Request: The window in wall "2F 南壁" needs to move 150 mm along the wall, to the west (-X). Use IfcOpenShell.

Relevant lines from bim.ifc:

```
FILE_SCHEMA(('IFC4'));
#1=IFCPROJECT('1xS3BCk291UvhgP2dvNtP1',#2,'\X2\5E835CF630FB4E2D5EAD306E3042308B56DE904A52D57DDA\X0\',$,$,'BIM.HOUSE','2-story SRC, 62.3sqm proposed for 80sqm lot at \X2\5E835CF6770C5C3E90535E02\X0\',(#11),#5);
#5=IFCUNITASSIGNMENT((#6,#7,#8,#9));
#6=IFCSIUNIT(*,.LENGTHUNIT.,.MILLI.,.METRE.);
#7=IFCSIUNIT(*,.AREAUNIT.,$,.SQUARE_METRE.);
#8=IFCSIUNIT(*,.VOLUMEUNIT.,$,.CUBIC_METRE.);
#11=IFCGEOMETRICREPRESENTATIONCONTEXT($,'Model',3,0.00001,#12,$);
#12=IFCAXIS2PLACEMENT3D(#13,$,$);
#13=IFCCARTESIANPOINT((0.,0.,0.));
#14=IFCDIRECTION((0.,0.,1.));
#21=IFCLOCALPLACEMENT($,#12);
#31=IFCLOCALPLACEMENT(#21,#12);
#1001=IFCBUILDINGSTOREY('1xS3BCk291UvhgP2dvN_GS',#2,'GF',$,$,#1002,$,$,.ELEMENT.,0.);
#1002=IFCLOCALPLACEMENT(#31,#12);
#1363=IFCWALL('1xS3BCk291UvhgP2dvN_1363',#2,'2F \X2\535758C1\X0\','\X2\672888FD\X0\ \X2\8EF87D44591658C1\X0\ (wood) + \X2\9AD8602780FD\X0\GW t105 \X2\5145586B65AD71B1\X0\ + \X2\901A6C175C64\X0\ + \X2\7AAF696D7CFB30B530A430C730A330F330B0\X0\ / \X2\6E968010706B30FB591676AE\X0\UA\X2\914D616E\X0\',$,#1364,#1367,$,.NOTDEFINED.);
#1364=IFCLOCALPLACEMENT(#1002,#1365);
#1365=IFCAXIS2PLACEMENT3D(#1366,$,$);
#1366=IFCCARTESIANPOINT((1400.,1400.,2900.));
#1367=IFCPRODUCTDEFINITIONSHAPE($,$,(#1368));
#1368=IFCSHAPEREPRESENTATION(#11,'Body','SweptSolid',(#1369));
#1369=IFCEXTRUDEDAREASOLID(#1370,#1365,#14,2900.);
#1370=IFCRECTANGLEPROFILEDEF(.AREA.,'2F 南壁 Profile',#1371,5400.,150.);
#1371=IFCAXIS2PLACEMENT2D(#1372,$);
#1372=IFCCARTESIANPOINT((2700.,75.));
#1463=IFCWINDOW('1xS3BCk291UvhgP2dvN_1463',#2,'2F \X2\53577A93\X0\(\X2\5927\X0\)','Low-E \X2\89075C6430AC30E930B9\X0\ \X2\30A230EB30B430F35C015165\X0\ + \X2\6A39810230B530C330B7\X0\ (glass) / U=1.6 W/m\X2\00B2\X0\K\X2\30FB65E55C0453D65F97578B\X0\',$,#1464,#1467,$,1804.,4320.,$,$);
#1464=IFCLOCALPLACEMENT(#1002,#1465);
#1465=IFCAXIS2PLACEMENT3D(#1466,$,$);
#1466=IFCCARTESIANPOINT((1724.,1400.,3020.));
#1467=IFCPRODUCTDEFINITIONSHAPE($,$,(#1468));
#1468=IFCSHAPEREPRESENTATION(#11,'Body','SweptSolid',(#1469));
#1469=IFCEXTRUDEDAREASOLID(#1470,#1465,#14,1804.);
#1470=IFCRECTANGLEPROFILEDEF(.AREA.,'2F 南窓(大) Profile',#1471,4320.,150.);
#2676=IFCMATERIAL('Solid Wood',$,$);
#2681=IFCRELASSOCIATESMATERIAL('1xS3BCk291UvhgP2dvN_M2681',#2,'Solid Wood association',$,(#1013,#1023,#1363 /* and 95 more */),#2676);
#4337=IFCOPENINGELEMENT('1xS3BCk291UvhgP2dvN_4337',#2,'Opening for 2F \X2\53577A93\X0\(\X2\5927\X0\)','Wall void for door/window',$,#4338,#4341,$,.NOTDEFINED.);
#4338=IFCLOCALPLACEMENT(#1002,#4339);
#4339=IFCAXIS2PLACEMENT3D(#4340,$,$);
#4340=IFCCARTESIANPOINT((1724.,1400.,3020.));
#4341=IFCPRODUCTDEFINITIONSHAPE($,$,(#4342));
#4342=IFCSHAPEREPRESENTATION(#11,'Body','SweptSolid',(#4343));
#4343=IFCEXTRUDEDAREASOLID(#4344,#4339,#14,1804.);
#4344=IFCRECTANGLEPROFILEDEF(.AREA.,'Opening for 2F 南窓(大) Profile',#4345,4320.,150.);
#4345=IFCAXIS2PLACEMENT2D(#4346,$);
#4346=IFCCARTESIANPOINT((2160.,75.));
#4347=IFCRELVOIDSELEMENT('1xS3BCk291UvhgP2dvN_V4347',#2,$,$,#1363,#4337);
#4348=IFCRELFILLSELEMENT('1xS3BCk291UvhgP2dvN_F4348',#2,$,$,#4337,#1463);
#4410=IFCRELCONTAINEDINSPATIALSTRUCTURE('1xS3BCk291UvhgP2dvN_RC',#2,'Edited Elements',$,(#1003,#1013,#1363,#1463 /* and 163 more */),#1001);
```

```python
import ifcopenshell
import ifcopenshell.api.geometry
import ifcopenshell.util.placement

model = ifcopenshell.open("bim.ifc")

window = model.by_guid("1xS3BCk291UvhgP2dvN_1463")
opening = window.FillsVoids[0].RelatingOpeningElement
wall = opening.VoidsElements[0].RelatingBuildingElement

wall_matrix = ifcopenshell.util.placement.get_local_placement(wall.ObjectPlacement)
shift = wall_matrix[:3, 0] * -150.0
before = ifcopenshell.util.placement.get_local_placement(window.ObjectPlacement)[:3, 3].copy()

# The window is not placed relative to its opening, so move both.
for product in (opening, window):
    matrix = ifcopenshell.util.placement.get_local_placement(product.ObjectPlacement)
    matrix[:3, 3] += shift
    ifcopenshell.api.geometry.edit_object_placement(model, product=product, matrix=matrix, is_si=False)

after = ifcopenshell.util.placement.get_local_placement(window.ObjectPlacement)[:3, 3]
print("window moved by", (after - before).round(3) + 0.0)

model.write("bim_edited.ifc")
```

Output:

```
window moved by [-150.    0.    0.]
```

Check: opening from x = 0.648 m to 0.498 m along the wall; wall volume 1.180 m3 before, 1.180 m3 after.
